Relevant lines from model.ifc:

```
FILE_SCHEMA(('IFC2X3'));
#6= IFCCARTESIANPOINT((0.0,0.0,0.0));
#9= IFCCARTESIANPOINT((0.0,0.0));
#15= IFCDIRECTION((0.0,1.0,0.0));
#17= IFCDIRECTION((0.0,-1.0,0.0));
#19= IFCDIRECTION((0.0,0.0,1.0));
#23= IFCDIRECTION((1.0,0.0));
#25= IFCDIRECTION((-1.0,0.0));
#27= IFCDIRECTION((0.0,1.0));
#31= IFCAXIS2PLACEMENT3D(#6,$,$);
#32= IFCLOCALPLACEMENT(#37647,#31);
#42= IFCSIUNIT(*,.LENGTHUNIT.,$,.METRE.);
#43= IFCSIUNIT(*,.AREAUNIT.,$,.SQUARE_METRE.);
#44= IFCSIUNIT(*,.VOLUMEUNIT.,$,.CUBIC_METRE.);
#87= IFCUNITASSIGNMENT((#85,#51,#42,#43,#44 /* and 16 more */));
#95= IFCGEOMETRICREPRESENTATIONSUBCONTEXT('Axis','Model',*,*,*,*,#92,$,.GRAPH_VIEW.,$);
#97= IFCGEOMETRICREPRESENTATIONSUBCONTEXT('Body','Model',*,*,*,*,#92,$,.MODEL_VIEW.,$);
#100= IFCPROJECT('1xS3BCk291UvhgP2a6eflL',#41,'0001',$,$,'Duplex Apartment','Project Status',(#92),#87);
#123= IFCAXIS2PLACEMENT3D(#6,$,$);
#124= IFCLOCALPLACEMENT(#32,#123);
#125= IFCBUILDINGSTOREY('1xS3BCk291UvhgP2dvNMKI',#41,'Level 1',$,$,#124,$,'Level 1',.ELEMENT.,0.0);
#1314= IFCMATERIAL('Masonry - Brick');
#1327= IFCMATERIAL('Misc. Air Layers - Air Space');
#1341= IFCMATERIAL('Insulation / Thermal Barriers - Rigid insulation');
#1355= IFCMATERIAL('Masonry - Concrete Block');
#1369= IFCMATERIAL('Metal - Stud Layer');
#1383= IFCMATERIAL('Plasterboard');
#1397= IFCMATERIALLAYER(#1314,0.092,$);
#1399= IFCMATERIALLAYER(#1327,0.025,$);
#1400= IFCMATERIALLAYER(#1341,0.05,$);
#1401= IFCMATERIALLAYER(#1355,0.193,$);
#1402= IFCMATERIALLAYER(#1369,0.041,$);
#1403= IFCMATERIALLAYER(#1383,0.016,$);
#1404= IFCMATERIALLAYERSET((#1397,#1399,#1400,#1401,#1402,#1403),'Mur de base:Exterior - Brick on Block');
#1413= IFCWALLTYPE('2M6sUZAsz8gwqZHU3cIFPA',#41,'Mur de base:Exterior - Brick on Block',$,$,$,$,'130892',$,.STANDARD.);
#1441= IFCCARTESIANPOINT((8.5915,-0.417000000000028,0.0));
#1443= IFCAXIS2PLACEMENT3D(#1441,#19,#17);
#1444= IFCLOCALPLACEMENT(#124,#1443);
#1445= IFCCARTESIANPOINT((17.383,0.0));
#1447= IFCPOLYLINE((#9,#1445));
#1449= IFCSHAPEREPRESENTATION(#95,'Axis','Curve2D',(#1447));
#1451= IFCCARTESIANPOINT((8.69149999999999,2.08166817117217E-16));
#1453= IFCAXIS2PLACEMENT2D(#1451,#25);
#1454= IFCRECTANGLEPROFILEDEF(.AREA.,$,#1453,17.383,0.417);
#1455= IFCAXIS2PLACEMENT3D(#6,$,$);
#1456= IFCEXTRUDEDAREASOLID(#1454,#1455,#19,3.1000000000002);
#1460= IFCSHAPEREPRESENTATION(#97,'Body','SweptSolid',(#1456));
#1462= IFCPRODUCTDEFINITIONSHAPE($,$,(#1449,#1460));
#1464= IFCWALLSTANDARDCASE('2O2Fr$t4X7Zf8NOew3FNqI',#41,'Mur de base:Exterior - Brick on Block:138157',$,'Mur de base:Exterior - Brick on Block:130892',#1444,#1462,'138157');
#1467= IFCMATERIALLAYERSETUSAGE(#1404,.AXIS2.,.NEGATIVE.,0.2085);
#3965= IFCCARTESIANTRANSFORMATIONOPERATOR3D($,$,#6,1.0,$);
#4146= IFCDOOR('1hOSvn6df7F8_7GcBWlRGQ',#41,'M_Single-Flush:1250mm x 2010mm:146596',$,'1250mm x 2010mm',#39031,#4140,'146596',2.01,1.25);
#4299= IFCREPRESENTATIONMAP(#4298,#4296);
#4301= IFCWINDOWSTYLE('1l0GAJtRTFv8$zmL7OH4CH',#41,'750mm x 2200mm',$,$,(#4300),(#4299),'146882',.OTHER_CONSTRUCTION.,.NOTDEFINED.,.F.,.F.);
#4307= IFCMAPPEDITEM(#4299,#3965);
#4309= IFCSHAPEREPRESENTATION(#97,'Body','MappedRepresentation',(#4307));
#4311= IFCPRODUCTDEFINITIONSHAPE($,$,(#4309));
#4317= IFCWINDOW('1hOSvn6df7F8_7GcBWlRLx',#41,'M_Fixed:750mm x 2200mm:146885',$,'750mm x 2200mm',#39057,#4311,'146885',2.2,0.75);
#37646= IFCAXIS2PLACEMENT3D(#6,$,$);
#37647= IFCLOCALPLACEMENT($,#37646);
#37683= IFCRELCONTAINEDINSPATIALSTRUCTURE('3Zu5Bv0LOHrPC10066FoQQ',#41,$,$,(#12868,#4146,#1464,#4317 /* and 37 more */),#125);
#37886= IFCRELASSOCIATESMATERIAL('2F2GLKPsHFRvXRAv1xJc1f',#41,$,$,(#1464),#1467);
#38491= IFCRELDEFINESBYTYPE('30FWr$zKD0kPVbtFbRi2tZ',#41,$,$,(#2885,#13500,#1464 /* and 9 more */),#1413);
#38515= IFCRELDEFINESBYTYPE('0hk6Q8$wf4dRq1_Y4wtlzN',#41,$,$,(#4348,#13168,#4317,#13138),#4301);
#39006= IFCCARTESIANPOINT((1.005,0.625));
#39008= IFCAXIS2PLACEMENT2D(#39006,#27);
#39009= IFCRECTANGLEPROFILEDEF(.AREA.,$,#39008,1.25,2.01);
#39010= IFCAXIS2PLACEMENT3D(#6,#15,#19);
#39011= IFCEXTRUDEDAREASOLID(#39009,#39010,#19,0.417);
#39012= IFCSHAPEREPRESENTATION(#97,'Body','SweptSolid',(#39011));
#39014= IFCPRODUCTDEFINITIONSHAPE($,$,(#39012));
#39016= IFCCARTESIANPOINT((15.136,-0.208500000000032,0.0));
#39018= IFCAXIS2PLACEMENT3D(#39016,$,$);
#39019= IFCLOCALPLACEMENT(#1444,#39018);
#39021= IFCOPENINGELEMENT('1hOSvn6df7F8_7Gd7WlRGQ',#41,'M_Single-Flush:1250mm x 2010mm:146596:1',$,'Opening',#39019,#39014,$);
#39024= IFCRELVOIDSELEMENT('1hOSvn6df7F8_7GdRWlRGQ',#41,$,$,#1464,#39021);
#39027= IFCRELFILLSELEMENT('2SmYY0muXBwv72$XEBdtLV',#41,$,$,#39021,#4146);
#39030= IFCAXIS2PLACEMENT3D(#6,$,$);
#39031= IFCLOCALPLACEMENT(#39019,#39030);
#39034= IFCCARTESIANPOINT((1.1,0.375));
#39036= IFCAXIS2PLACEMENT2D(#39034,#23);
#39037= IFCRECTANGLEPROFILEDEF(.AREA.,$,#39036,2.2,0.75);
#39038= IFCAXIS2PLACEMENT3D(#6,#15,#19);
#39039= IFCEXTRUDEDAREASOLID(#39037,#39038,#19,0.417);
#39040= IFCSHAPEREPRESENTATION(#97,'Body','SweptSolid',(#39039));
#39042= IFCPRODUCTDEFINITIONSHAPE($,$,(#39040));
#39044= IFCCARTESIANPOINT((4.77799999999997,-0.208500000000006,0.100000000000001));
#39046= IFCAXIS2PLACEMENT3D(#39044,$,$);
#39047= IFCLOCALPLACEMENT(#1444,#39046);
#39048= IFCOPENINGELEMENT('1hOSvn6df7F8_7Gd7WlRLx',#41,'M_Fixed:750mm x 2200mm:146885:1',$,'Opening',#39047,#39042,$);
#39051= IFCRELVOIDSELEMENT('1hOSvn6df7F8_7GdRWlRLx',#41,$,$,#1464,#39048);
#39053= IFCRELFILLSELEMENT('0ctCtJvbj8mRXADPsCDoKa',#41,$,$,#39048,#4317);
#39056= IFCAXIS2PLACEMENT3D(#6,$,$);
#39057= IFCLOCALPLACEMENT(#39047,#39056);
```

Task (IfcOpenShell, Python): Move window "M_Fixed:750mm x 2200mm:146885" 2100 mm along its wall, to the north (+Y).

```python
import ifcopenshell
import ifcopenshell.api.geometry
import ifcopenshell.util.placement

model = ifcopenshell.open("model.ifc")

window = model.by_guid("1hOSvn6df7F8_7GcBWlRLx")
opening = window.FillsVoids[0].RelatingOpeningElement
wall = opening.VoidsElements[0].RelatingBuildingElement

wall_matrix = ifcopenshell.util.placement.get_local_placement(wall.ObjectPlacement)
shift = wall_matrix[:3, 0] * -2.1
before = ifcopenshell.util.placement.get_local_placement(window.ObjectPlacement)[:3, 3].copy()

# The window is placed relative to its opening, so it follows when the opening moves.
matrix = ifcopenshell.util.placement.get_local_placement(opening.ObjectPlacement)
matrix[:3, 3] += shift
ifcopenshell.api.geometry.edit_object_placement(
    model, product=opening, matrix=matrix, is_si=False, should_transform_children=True
)

after = ifcopenshell.util.placement.get_local_placement(window.ObjectPlacement)[:3, 3]
print("window moved by", (after - before).round(3) + 0.0)

model.write("model-out.ifc")
```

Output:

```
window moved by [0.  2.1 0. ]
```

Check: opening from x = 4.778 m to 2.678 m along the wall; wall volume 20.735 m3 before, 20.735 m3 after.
